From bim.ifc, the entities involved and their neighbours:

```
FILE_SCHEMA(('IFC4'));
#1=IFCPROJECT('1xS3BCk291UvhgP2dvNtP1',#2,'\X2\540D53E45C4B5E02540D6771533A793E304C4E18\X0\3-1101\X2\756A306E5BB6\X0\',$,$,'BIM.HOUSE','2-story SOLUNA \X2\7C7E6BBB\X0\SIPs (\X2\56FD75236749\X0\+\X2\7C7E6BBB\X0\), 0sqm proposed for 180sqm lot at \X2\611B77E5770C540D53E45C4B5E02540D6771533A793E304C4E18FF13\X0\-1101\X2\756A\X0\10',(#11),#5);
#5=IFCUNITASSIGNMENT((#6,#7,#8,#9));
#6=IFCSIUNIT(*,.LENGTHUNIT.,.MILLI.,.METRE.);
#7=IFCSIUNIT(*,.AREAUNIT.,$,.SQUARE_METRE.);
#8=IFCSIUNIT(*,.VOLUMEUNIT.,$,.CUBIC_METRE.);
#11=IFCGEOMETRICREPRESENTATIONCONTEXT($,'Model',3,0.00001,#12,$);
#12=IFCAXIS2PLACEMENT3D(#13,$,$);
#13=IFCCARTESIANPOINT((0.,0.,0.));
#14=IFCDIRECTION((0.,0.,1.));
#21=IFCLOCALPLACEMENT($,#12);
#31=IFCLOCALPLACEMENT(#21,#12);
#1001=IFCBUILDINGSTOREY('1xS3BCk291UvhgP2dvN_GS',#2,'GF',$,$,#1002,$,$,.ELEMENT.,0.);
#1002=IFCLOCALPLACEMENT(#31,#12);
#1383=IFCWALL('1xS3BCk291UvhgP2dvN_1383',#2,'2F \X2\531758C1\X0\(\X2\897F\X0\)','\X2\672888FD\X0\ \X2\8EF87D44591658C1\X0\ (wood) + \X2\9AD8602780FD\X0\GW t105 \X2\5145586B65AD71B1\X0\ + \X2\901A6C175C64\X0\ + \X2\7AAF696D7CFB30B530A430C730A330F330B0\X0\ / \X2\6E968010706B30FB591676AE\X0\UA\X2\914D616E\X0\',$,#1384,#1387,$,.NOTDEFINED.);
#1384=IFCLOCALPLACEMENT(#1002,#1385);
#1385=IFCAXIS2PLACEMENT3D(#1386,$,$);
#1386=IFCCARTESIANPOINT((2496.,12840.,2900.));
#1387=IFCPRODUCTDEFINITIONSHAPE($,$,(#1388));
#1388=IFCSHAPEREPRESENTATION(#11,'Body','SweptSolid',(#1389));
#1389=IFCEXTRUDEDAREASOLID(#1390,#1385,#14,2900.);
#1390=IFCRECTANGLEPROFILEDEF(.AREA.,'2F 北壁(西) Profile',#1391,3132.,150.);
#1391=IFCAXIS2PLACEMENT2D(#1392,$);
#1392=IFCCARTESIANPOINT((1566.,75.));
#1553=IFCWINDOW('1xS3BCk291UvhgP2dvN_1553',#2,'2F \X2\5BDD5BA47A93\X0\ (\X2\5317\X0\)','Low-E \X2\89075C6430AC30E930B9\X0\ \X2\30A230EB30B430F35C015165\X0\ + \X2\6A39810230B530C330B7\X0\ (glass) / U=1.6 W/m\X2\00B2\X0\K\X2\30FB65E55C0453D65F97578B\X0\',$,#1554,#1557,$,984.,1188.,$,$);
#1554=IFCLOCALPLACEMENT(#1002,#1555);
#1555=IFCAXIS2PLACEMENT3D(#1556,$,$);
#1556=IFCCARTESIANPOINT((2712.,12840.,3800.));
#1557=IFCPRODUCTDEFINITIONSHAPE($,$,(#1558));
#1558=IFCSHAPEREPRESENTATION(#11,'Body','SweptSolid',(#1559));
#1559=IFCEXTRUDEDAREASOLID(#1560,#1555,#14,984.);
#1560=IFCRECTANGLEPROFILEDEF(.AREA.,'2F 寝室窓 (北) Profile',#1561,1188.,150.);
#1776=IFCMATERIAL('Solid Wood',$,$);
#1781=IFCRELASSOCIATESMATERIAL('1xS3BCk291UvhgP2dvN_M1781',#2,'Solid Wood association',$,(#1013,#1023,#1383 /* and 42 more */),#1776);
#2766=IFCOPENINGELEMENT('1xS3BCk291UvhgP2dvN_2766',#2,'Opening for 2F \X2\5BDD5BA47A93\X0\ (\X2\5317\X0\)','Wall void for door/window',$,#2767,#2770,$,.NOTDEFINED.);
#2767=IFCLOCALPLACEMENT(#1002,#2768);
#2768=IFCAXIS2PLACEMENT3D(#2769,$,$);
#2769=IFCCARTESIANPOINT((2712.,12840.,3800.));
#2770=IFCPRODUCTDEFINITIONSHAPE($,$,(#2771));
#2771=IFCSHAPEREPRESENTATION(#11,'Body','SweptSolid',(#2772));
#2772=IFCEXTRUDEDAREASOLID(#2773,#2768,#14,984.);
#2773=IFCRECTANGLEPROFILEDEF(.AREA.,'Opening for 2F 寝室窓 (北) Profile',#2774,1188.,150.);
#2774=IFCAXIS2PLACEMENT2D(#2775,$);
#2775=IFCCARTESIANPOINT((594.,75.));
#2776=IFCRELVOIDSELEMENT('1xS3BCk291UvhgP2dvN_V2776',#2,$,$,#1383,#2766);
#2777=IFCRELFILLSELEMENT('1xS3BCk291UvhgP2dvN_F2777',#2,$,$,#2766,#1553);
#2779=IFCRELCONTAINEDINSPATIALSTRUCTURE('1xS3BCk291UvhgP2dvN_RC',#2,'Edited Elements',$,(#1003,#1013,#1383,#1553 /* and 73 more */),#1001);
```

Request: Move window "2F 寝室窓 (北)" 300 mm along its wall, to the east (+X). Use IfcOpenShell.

```python
import ifcopenshell
import ifcopenshell.api.geometry
import ifcopenshell.util.placement

model = ifcopenshell.open("bim.ifc")

window = model.by_id(1553)
opening = window.FillsVoids[0].RelatingOpeningElement
wall = opening.VoidsElements[0].RelatingBuildingElement

wall_matrix = ifcopenshell.util.placement.get_local_placement(wall.ObjectPlacement)
shift = wall_matrix[:3, 0] * 300.0
before = ifcopenshell.util.placement.get_local_placement(window.ObjectPlacement)[:3, 3].copy()

# The window is not placed relative to its opening, so move both.
for product in (opening, window):
    matrix = ifcopenshell.util.placement.get_local_placement(product.ObjectPlacement)
    matrix[:3, 3] += shift
    ifcopenshell.api.geometry.edit_object_placement(model, product=product, matrix=matrix, is_si=False)

after = ifcopenshell.util.placement.get_local_placement(window.ObjectPlacement)[:3, 3]
print("window moved by", (after - before).round(3) + 0.0)

model.write("bim-out.ifc")
```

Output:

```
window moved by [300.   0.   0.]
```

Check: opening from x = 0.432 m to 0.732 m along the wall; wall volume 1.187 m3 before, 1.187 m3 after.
